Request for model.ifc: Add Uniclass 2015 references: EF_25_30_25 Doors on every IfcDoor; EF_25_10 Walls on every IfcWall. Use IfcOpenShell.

First a look at what the model holds.

```python
import ifcopenshell

model = ifcopenshell.open("model.ifc")
print(model.schema)
print("classifications:", [c.Name for c in model.by_type("IfcClassification")])
for ifc_class in ("IfcDoor", "IfcRoof", "IfcStair", "IfcWall", "IfcWindow"):
    print(ifc_class, len(model.by_type(ifc_class)))
```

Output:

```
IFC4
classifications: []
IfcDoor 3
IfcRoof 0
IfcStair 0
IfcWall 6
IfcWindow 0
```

```python
import ifcopenshell
import ifcopenshell.api.classification

model = ifcopenshell.open("model.ifc")

system = ifcopenshell.api.classification.add_classification(model, classification="Uniclass 2015")

codes = {
    "IfcDoor": ("EF_25_30_25", "Doors"),
    "IfcWall": ("EF_25_10", "Walls"),
}
for ifc_class, (code, name) in codes.items():
    products = model.by_type(ifc_class)
    ifcopenshell.api.classification.add_reference(
        model, products=products, classification=system, identification=code, name=name
    )
    print(code, len(products))

model.write("model_v2.ifc")
```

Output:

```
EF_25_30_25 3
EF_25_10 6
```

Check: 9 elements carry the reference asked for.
